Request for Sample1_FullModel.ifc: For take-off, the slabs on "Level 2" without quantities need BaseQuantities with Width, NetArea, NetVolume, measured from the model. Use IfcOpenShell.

First a look at what the model holds.

```python
import ifcopenshell
import ifcopenshell.util.element
import ifcopenshell.util.unit

model = ifcopenshell.open("Sample1_FullModel.ifc")
print(model.schema)
for unit_type in ("LENGTHUNIT", "AREAUNIT", "VOLUMEUNIT"):
    print(unit_type, ifcopenshell.util.unit.calculate_unit_scale(model, unit_type))
storey = next(s for s in model.by_type("IfcBuildingStorey") if s.Name == "Level 2")
slabs = [e for e in ifcopenshell.util.element.get_decomposition(storey) if e.is_a("IfcSlab")]
for e in sorted(slabs, key=lambda e: e.id()):
    print(e.id(), e.is_a(), e.Name, list(ifcopenshell.util.element.get_psets(e, qtos_only=True)), sep=" | ")
```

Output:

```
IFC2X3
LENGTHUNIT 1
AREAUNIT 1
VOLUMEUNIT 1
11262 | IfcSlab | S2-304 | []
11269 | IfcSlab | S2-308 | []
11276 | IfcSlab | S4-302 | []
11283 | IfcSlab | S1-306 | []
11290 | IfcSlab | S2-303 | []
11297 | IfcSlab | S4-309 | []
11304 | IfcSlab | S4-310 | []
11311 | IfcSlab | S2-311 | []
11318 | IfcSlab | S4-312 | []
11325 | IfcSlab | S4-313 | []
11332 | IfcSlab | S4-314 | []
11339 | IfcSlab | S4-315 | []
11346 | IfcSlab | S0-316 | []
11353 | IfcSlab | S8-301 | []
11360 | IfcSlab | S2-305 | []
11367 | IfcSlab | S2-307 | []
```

```python
import ifcopenshell
import ifcopenshell.api.pset
import ifcopenshell.geom
import ifcopenshell.util.element
import ifcopenshell.util.shape
import ifcopenshell.util.unit

model = ifcopenshell.open("Sample1_FullModel.ifc")
unit_scale = ifcopenshell.util.unit.calculate_unit_scale(model)
area_scale = ifcopenshell.util.unit.calculate_unit_scale(model, "AREAUNIT")
volume_scale = ifcopenshell.util.unit.calculate_unit_scale(model, "VOLUMEUNIT")
settings = ifcopenshell.geom.settings()

storey = next(s for s in model.by_type("IfcBuildingStorey") if s.Name == "Level 2")
slabs = [e for e in ifcopenshell.util.element.get_decomposition(storey) if e.is_a("IfcSlab")]

for e in sorted(slabs, key=lambda e: e.id()):
    if ifcopenshell.util.element.get_psets(e, qtos_only=True, should_inherit=False):
        continue
    # Geometry comes back in metres, in the element's own axes.
    shape = ifcopenshell.geom.create_shape(settings, e)
    values = {
        "Width": ifcopenshell.util.shape.get_z(shape.geometry) / unit_scale,
        "NetArea": ifcopenshell.util.shape.get_footprint_area(shape.geometry) / area_scale,
        "NetVolume": ifcopenshell.util.shape.get_volume(shape.geometry) / volume_scale,
    }
    qto = ifcopenshell.api.pset.add_qto(model, product=e, name="BaseQuantities")
    ifcopenshell.api.pset.edit_qto(model, qto=qto, properties=values)
    print(e.id(), {k: round(v, 3) for k, v in values.items()})

model.write("Sample1_FullModel_v2.ifc")
```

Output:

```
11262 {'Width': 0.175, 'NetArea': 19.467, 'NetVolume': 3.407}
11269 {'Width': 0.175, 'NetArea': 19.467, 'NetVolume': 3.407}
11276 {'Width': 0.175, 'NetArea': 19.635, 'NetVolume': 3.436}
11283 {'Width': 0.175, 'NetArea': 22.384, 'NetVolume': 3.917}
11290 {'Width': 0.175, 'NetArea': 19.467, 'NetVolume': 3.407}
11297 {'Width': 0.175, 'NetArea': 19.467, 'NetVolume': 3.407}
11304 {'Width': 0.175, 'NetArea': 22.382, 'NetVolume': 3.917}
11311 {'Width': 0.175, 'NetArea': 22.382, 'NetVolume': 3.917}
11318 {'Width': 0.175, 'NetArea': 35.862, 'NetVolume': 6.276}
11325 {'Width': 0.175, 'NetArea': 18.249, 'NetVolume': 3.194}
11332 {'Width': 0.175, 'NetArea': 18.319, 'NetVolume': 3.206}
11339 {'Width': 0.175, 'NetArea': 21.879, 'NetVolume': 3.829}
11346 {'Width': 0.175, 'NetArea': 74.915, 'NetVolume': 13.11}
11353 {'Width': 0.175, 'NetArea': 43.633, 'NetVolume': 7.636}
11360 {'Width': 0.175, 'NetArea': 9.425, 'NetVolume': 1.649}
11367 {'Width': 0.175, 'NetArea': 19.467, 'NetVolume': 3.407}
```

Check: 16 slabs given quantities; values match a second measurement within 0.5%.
